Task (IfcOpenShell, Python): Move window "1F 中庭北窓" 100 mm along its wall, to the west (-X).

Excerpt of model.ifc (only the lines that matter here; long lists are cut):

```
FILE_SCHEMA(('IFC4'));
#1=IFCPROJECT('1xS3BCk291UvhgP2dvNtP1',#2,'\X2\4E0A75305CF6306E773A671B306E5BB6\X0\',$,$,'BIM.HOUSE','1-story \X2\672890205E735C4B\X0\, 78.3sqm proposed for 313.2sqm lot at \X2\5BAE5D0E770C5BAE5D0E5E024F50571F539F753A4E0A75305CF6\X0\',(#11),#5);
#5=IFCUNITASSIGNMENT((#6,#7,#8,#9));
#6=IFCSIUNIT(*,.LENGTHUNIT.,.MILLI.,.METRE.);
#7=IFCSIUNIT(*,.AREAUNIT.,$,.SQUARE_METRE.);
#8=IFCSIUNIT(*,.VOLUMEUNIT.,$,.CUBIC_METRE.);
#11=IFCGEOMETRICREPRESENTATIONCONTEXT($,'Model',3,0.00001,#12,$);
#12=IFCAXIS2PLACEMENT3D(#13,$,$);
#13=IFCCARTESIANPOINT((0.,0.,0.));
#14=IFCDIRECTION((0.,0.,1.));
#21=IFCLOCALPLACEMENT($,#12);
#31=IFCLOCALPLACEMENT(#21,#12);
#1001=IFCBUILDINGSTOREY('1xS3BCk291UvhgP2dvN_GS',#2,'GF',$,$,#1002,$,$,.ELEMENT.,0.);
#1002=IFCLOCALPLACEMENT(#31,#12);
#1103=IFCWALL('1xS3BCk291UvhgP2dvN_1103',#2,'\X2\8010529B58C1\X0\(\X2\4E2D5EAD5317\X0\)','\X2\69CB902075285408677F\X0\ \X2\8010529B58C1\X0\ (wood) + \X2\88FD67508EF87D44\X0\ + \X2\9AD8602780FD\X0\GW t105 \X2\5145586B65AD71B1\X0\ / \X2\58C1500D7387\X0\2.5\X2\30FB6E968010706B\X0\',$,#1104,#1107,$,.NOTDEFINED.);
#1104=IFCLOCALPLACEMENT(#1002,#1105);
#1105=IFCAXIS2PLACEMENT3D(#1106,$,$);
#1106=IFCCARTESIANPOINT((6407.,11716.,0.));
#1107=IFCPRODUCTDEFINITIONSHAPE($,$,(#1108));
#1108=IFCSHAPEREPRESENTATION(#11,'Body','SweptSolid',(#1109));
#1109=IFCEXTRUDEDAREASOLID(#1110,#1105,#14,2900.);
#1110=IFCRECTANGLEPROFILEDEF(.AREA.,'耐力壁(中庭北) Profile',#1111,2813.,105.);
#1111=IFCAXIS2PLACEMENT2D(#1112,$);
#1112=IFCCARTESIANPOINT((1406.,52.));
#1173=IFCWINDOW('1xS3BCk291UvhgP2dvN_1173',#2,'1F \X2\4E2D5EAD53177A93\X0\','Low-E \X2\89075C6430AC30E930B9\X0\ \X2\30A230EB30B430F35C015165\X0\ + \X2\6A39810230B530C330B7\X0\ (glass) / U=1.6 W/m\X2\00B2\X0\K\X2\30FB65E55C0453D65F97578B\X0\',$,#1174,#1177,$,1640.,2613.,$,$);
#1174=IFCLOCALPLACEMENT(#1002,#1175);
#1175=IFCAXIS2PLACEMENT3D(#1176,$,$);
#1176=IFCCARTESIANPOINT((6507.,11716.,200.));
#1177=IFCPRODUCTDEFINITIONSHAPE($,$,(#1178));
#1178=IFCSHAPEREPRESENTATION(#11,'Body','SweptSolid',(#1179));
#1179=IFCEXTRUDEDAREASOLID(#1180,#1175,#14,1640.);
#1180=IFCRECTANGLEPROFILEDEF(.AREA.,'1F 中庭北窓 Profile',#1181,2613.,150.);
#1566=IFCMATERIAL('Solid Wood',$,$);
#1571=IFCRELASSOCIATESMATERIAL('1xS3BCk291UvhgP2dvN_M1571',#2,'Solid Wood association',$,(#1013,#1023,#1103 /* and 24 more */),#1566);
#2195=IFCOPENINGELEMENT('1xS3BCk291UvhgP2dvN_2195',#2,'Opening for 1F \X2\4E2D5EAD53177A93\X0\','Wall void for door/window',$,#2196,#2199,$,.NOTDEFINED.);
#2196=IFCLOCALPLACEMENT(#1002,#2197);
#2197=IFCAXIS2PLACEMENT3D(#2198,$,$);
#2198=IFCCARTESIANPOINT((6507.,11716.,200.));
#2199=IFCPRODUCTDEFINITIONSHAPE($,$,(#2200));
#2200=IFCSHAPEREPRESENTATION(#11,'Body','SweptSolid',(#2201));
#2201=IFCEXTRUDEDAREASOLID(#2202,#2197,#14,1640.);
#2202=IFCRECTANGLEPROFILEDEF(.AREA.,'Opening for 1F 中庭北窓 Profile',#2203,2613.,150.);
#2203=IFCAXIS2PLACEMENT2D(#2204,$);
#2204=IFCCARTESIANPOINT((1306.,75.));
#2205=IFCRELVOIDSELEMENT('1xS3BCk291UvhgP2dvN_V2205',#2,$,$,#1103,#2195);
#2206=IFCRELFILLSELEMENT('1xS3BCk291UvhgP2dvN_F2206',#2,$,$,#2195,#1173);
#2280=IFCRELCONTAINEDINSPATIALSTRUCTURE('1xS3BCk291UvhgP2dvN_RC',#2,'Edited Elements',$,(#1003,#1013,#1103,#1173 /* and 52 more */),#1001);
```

```python
import ifcopenshell
import ifcopenshell.api.geometry
import ifcopenshell.util.placement
import ifcopenshell.util.unit

model = ifcopenshell.open("model.ifc")
unit_scale = ifcopenshell.util.unit.calculate_unit_scale(model)

window = model.by_guid("1xS3BCk291UvhgP2dvN_1173")
opening = window.FillsVoids[0].RelatingOpeningElement
wall = opening.VoidsElements[0].RelatingBuildingElement

wall_matrix = ifcopenshell.util.placement.get_local_placement(wall.ObjectPlacement)
shift = wall_matrix[:3, 0] * -0.1 / unit_scale
before = ifcopenshell.util.placement.get_local_placement(window.ObjectPlacement)[:3, 3].copy()

# The window is not placed relative to its opening, so move both.
for product in (opening, window):
    matrix = ifcopenshell.util.placement.get_local_placement(product.ObjectPlacement)
    matrix[:3, 3] += shift
    ifcopenshell.api.geometry.edit_object_placement(model, product=product, matrix=matrix, is_si=False)

after = ifcopenshell.util.placement.get_local_placement(window.ObjectPlacement)[:3, 3]
print("window moved by", (after - before).round(3) + 0.0)

model.write("model_v2.ifc")
```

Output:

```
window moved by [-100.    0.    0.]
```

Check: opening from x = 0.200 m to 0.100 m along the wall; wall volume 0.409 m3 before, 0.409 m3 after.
